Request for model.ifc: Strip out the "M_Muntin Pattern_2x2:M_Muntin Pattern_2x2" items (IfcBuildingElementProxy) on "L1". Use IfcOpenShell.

First a look at what the model holds.

```python
import ifcopenshell
import ifcopenshell.util.element

model = ifcopenshell.open("model.ifc")
print(model.schema)
storey = next(s for s in model.by_type("IfcBuildingStorey") if s.Name == "L1")
proxies = [e for e in ifcopenshell.util.element.get_decomposition(storey) if e.is_a("IfcBuildingElementProxy")]
seen = {}
for e in proxies:
    element_type = ifcopenshell.util.element.get_type(e)
    name = element_type.Name if element_type not in (None, e) else None
    seen[name] = seen.get(name, 0) + 1
for name, count in sorted(seen.items(), key=str):
    print(count, "x", name)
```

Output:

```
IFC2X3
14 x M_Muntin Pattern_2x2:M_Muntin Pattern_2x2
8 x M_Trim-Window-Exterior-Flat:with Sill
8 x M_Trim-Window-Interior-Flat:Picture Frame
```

```python
import ifcopenshell
import ifcopenshell.api.root
import ifcopenshell.util.element

model = ifcopenshell.open("model.ifc")

storey = next(s for s in model.by_type("IfcBuildingStorey") if s.Name == "L1")
proxies = [e for e in ifcopenshell.util.element.get_decomposition(storey) if e.is_a("IfcBuildingElementProxy")]
targets = [e for e in proxies if (t := ifcopenshell.util.element.get_type(e)) not in (None, e) and t.Name == "M_Muntin Pattern_2x2:M_Muntin Pattern_2x2"]

for e in targets:
    ifcopenshell.api.root.remove_product(model, product=e)
print(len(targets), "removed")

model.write("model_rev.ifc")
```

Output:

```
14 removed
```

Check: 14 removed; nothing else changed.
